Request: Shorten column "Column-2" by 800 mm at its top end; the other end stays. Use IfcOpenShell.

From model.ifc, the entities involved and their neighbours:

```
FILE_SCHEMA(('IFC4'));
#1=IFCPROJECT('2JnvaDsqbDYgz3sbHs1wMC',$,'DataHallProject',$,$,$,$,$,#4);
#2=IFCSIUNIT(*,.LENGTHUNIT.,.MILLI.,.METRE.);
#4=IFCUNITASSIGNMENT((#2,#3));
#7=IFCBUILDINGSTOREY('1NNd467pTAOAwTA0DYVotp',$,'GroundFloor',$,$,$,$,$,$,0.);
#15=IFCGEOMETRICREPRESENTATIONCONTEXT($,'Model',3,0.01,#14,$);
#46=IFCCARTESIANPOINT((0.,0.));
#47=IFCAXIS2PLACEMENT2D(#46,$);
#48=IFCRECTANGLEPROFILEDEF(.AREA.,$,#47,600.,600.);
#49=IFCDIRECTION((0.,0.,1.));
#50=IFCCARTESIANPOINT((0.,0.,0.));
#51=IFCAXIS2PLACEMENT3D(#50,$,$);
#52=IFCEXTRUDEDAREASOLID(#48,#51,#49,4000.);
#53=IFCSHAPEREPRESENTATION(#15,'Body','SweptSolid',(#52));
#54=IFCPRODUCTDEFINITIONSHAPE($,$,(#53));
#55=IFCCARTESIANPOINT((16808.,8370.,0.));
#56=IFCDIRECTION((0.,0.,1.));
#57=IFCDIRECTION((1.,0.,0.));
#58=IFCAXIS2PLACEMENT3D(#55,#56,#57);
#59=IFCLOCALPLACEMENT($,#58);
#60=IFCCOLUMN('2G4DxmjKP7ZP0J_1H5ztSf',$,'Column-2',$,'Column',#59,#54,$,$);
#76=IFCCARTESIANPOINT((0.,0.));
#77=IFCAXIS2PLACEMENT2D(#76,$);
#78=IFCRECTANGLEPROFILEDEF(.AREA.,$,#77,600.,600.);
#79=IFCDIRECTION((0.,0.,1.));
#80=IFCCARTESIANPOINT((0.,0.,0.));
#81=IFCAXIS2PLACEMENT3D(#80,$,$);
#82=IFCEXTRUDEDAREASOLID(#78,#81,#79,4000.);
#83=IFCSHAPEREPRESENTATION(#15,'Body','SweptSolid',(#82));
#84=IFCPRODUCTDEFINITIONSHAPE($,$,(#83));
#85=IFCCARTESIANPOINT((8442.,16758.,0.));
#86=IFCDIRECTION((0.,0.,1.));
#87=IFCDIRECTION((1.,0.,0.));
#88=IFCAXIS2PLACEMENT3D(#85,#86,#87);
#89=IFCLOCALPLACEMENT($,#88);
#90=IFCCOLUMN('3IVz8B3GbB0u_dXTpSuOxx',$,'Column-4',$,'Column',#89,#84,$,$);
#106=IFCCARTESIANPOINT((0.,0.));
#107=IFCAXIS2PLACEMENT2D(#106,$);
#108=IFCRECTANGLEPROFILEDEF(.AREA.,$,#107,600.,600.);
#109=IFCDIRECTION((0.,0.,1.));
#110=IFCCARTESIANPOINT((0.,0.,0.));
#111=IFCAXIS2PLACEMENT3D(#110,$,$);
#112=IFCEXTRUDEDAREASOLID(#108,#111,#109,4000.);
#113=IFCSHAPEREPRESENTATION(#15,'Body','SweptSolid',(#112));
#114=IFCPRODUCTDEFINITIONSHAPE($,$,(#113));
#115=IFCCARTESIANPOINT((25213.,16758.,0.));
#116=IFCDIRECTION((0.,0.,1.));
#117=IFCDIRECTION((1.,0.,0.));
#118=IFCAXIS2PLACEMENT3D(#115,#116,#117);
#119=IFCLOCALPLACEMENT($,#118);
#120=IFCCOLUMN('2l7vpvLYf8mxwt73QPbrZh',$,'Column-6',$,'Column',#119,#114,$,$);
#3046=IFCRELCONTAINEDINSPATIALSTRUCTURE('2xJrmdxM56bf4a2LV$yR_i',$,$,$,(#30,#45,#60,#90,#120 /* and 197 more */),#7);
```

```python
import ifcopenshell
import ifcopenshell.util.unit

model = ifcopenshell.open("model.ifc")
unit_scale = ifcopenshell.util.unit.calculate_unit_scale(model)

member = model.by_id(60)
change = -0.8 / unit_scale

# The extrusion runs towards the end named, so only its depth changes.
body = next(r for r in member.Representation.Representations if r.RepresentationIdentifier == "Body")
solid = body.Items[0]
old_length = solid.Depth
solid.Depth += change

print(f"length {old_length:g} -> {solid.Depth:g}")

model.write("model_updated.ifc")
```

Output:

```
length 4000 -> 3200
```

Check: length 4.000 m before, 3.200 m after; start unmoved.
